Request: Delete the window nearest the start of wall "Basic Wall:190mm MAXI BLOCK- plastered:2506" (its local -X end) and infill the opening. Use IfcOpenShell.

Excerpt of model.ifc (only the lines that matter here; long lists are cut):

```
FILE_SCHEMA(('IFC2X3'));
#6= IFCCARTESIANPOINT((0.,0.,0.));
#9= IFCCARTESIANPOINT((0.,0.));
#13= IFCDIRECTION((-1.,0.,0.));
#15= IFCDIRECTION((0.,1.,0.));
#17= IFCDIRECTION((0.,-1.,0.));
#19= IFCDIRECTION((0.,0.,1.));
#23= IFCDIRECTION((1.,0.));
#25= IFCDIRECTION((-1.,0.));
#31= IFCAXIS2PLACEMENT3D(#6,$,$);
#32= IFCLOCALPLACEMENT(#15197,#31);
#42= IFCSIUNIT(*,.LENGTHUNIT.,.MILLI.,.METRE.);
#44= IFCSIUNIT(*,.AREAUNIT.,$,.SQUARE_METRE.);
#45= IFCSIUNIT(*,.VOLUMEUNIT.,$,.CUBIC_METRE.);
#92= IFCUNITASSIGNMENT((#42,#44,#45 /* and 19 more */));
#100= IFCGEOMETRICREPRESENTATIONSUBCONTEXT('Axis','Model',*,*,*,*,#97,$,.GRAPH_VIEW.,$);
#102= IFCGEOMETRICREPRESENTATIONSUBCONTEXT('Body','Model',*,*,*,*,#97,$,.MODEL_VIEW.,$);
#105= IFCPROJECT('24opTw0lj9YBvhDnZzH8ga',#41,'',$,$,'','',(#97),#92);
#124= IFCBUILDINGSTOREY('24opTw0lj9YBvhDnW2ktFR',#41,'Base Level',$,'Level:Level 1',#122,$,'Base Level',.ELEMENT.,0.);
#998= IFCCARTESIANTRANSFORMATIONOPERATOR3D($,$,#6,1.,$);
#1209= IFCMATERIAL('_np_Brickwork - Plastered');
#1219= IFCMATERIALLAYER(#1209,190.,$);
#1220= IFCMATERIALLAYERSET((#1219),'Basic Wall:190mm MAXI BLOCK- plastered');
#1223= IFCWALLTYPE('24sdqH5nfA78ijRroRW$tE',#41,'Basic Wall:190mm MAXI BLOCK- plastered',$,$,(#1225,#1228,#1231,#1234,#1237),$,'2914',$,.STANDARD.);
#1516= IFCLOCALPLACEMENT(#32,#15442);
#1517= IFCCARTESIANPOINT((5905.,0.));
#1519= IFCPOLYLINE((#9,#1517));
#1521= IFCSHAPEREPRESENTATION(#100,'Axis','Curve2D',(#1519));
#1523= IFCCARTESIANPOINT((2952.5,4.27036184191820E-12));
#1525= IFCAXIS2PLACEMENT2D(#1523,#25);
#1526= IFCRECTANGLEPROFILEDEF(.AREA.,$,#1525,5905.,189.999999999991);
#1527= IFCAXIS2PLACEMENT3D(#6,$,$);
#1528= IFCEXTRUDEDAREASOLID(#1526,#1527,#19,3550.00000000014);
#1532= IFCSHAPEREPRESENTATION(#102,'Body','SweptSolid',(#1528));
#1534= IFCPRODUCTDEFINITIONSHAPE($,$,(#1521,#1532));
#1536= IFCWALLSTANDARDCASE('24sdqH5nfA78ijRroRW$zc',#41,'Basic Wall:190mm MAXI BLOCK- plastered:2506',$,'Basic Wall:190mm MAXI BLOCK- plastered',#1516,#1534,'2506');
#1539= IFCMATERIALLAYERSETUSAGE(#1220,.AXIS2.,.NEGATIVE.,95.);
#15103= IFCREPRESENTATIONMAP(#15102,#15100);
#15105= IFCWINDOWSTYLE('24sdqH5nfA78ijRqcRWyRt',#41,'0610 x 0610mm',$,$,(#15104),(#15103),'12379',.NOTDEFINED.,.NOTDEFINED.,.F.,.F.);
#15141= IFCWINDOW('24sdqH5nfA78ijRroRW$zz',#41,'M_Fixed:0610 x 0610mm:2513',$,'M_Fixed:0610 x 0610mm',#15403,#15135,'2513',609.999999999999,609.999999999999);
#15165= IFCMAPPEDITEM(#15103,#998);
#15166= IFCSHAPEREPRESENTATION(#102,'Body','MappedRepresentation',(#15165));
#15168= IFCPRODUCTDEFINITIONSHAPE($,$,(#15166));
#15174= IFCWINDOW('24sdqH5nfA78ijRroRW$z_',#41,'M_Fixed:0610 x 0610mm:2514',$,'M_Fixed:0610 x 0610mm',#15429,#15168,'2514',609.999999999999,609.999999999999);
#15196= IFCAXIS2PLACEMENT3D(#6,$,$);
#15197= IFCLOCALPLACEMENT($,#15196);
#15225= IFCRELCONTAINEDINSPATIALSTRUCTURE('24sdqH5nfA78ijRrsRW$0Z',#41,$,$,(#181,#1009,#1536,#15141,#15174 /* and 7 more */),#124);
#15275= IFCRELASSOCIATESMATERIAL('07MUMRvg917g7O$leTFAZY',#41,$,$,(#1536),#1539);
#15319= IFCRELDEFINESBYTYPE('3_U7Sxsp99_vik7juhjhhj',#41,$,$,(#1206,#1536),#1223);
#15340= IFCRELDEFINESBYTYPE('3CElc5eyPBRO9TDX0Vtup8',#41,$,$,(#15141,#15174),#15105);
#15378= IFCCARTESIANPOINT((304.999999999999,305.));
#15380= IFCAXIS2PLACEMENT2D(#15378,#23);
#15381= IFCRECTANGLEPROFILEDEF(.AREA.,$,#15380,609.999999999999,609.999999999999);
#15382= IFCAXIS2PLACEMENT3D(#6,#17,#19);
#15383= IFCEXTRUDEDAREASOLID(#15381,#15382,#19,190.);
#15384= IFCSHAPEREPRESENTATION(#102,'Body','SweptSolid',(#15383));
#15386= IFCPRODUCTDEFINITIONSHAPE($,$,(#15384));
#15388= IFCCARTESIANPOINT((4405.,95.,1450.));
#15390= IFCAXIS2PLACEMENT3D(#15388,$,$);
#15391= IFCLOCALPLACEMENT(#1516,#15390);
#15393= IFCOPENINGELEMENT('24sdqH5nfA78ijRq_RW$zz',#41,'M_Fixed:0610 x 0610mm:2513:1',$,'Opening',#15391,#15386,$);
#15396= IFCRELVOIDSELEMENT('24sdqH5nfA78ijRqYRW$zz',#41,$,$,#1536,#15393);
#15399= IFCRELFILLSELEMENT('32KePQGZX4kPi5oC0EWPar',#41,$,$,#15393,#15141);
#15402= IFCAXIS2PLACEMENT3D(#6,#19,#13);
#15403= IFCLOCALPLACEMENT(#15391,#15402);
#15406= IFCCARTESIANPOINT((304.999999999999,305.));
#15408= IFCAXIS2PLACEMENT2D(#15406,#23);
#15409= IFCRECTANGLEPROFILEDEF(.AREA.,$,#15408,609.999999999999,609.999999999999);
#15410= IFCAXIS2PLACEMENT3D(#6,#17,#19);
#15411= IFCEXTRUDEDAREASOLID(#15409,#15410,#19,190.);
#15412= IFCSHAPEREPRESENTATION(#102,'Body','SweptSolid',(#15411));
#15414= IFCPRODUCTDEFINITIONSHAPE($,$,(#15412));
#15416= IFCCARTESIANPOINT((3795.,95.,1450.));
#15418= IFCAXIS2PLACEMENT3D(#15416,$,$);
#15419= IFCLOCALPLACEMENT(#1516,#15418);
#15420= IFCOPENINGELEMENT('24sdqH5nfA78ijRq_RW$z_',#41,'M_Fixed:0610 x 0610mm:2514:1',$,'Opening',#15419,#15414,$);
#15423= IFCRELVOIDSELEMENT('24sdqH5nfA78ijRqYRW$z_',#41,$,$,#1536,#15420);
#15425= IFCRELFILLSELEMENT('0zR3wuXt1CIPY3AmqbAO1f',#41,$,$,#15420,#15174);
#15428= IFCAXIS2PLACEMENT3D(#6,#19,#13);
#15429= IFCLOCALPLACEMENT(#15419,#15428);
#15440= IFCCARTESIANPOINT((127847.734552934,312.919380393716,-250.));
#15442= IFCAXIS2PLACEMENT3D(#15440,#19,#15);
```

```python
import ifcopenshell
import ifcopenshell.api.feature
import ifcopenshell.api.root
import ifcopenshell.geom
import ifcopenshell.util.shape

model = ifcopenshell.open("model.ifc")
settings = ifcopenshell.geom.settings()


def volume(element):
    """Net volume in cubic metres, openings subtracted."""
    shape = ifcopenshell.geom.create_shape(settings, element)
    return ifcopenshell.util.shape.get_volume(shape.geometry)


window = model.by_guid("24sdqH5nfA78ijRroRW$z_")
opening = window.FillsVoids[0].RelatingOpeningElement
wall = opening.VoidsElements[0].RelatingBuildingElement
before = volume(wall)

ifcopenshell.api.root.remove_product(model, product=window)
ifcopenshell.api.feature.remove_feature(model, feature=opening)

after = volume(wall)

print(f"wall volume {before:.3f} -> {after:.3f} m3")

model.write("model_rev.ifc")
```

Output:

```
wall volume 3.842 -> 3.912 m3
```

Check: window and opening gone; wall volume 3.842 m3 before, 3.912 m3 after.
